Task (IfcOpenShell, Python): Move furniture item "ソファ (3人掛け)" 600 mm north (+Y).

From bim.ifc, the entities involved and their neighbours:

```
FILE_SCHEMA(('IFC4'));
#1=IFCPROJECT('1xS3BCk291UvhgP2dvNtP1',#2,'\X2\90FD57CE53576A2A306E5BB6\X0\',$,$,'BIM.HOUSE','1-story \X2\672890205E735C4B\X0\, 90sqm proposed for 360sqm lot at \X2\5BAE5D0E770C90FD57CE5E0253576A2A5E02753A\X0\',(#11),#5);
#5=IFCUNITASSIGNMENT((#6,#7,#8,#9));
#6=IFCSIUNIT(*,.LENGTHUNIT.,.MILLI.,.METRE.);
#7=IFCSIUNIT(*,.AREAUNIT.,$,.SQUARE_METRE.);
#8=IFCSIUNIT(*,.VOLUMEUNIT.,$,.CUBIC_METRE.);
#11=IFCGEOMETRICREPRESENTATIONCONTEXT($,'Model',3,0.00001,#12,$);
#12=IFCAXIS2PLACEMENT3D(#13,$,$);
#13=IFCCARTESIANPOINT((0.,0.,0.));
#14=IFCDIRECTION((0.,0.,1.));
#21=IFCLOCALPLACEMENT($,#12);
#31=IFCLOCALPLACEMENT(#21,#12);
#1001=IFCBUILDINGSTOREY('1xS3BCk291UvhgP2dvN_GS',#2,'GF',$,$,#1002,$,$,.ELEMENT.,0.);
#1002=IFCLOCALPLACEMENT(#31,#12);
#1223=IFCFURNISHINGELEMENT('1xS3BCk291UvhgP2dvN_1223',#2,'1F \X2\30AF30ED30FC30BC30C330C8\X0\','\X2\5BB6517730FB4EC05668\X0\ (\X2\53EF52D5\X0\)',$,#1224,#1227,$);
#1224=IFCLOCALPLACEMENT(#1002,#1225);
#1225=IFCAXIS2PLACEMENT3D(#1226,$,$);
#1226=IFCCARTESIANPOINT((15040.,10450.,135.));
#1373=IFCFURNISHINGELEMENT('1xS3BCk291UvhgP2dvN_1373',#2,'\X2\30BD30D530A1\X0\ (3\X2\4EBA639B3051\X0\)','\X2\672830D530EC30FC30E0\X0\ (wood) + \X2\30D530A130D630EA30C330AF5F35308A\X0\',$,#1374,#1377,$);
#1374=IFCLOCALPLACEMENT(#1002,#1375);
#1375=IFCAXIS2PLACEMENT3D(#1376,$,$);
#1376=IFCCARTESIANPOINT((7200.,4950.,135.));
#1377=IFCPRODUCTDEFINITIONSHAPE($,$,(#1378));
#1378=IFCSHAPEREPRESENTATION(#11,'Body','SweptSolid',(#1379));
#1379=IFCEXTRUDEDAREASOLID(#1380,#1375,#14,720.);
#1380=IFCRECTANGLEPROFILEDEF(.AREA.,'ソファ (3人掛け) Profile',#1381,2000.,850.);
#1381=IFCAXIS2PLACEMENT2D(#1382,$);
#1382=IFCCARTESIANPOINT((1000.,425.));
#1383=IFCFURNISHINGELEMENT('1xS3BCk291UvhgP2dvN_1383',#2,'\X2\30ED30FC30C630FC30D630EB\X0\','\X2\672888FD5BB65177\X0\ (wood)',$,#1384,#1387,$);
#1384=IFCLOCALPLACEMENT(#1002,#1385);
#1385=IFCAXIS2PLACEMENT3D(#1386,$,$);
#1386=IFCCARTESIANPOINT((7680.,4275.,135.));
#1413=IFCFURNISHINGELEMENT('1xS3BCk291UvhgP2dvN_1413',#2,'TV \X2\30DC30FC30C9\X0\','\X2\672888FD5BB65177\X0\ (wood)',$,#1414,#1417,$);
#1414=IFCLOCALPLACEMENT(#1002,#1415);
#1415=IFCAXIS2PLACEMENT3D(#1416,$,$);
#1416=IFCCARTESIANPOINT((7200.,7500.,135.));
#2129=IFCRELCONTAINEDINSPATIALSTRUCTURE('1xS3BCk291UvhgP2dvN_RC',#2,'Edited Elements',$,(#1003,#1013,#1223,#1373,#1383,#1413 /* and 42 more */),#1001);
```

```python
import ifcopenshell
import ifcopenshell.api.geometry
import ifcopenshell.util.placement
import ifcopenshell.util.unit

model = ifcopenshell.open("bim.ifc")
unit_scale = ifcopenshell.util.unit.calculate_unit_scale(model)

item = model.by_guid("1xS3BCk291UvhgP2dvN_1373")
matrix = ifcopenshell.util.placement.get_local_placement(item.ObjectPlacement)
matrix[1, 3] += 0.6 / unit_scale
ifcopenshell.api.geometry.edit_object_placement(model, product=item, matrix=matrix, is_si=False)

print(ifcopenshell.util.placement.get_local_placement(item.ObjectPlacement).round(3) + 0.0)

model.write("bim_rev.ifc")
```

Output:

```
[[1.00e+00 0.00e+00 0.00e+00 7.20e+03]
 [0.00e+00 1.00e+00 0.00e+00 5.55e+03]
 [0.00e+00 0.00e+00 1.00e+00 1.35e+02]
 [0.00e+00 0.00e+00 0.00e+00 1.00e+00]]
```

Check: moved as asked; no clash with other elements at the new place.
